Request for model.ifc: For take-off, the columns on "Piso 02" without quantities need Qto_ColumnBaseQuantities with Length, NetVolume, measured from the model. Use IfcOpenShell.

First a look at what the model holds.

```python
import ifcopenshell
import ifcopenshell.util.element
import ifcopenshell.util.unit

model = ifcopenshell.open("model.ifc")
print(model.schema)
for unit_type in ("LENGTHUNIT", "AREAUNIT", "VOLUMEUNIT"):
    print(unit_type, ifcopenshell.util.unit.calculate_unit_scale(model, unit_type))
storey = next(s for s in model.by_type("IfcBuildingStorey") if s.Name == "Piso 02")
columns = [e for e in ifcopenshell.util.element.get_decomposition(storey) if e.is_a("IfcColumn")]
for e in sorted(columns, key=lambda e: e.id()):
    print(e.id(), e.is_a(), e.Name, list(ifcopenshell.util.element.get_psets(e, qtos_only=True)), sep=" | ")
```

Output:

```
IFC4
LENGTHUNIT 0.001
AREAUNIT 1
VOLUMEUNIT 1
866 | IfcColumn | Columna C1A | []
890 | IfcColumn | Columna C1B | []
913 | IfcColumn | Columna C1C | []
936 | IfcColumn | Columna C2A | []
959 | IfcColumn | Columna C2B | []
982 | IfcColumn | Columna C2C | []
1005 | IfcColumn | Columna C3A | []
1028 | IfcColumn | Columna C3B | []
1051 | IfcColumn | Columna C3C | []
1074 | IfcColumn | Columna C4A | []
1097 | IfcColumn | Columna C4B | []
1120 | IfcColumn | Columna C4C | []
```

```python
import ifcopenshell
import ifcopenshell.api.pset
import ifcopenshell.geom
import ifcopenshell.util.element
import ifcopenshell.util.shape
import ifcopenshell.util.unit

model = ifcopenshell.open("model.ifc")
unit_scale = ifcopenshell.util.unit.calculate_unit_scale(model)
volume_scale = ifcopenshell.util.unit.calculate_unit_scale(model, "VOLUMEUNIT")
settings = ifcopenshell.geom.settings()

storey = next(s for s in model.by_type("IfcBuildingStorey") if s.Name == "Piso 02")
columns = [e for e in ifcopenshell.util.element.get_decomposition(storey) if e.is_a("IfcColumn")]

for e in sorted(columns, key=lambda e: e.id()):
    if ifcopenshell.util.element.get_psets(e, qtos_only=True, should_inherit=False):
        continue
    # Geometry comes back in metres, in the element's own axes.
    shape = ifcopenshell.geom.create_shape(settings, e)
    values = {
        "Length": ifcopenshell.util.shape.get_z(shape.geometry) / unit_scale,
        "NetVolume": ifcopenshell.util.shape.get_volume(shape.geometry) / volume_scale,
    }
    qto = ifcopenshell.api.pset.add_qto(model, product=e, name="Qto_ColumnBaseQuantities")
    ifcopenshell.api.pset.edit_qto(model, qto=qto, properties=values)
    print(e.id(), {k: round(v, 3) for k, v in values.items()})

model.write("model_v2.ifc")
```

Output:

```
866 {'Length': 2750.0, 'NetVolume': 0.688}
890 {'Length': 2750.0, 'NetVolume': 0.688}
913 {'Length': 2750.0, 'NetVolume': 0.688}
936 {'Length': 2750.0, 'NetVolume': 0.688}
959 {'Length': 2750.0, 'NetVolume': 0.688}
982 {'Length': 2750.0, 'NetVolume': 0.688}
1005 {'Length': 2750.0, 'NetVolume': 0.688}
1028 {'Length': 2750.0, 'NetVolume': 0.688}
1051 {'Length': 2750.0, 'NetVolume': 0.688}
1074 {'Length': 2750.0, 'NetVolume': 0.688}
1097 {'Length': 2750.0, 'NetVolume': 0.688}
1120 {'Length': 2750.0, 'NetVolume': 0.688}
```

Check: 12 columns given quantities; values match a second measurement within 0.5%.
